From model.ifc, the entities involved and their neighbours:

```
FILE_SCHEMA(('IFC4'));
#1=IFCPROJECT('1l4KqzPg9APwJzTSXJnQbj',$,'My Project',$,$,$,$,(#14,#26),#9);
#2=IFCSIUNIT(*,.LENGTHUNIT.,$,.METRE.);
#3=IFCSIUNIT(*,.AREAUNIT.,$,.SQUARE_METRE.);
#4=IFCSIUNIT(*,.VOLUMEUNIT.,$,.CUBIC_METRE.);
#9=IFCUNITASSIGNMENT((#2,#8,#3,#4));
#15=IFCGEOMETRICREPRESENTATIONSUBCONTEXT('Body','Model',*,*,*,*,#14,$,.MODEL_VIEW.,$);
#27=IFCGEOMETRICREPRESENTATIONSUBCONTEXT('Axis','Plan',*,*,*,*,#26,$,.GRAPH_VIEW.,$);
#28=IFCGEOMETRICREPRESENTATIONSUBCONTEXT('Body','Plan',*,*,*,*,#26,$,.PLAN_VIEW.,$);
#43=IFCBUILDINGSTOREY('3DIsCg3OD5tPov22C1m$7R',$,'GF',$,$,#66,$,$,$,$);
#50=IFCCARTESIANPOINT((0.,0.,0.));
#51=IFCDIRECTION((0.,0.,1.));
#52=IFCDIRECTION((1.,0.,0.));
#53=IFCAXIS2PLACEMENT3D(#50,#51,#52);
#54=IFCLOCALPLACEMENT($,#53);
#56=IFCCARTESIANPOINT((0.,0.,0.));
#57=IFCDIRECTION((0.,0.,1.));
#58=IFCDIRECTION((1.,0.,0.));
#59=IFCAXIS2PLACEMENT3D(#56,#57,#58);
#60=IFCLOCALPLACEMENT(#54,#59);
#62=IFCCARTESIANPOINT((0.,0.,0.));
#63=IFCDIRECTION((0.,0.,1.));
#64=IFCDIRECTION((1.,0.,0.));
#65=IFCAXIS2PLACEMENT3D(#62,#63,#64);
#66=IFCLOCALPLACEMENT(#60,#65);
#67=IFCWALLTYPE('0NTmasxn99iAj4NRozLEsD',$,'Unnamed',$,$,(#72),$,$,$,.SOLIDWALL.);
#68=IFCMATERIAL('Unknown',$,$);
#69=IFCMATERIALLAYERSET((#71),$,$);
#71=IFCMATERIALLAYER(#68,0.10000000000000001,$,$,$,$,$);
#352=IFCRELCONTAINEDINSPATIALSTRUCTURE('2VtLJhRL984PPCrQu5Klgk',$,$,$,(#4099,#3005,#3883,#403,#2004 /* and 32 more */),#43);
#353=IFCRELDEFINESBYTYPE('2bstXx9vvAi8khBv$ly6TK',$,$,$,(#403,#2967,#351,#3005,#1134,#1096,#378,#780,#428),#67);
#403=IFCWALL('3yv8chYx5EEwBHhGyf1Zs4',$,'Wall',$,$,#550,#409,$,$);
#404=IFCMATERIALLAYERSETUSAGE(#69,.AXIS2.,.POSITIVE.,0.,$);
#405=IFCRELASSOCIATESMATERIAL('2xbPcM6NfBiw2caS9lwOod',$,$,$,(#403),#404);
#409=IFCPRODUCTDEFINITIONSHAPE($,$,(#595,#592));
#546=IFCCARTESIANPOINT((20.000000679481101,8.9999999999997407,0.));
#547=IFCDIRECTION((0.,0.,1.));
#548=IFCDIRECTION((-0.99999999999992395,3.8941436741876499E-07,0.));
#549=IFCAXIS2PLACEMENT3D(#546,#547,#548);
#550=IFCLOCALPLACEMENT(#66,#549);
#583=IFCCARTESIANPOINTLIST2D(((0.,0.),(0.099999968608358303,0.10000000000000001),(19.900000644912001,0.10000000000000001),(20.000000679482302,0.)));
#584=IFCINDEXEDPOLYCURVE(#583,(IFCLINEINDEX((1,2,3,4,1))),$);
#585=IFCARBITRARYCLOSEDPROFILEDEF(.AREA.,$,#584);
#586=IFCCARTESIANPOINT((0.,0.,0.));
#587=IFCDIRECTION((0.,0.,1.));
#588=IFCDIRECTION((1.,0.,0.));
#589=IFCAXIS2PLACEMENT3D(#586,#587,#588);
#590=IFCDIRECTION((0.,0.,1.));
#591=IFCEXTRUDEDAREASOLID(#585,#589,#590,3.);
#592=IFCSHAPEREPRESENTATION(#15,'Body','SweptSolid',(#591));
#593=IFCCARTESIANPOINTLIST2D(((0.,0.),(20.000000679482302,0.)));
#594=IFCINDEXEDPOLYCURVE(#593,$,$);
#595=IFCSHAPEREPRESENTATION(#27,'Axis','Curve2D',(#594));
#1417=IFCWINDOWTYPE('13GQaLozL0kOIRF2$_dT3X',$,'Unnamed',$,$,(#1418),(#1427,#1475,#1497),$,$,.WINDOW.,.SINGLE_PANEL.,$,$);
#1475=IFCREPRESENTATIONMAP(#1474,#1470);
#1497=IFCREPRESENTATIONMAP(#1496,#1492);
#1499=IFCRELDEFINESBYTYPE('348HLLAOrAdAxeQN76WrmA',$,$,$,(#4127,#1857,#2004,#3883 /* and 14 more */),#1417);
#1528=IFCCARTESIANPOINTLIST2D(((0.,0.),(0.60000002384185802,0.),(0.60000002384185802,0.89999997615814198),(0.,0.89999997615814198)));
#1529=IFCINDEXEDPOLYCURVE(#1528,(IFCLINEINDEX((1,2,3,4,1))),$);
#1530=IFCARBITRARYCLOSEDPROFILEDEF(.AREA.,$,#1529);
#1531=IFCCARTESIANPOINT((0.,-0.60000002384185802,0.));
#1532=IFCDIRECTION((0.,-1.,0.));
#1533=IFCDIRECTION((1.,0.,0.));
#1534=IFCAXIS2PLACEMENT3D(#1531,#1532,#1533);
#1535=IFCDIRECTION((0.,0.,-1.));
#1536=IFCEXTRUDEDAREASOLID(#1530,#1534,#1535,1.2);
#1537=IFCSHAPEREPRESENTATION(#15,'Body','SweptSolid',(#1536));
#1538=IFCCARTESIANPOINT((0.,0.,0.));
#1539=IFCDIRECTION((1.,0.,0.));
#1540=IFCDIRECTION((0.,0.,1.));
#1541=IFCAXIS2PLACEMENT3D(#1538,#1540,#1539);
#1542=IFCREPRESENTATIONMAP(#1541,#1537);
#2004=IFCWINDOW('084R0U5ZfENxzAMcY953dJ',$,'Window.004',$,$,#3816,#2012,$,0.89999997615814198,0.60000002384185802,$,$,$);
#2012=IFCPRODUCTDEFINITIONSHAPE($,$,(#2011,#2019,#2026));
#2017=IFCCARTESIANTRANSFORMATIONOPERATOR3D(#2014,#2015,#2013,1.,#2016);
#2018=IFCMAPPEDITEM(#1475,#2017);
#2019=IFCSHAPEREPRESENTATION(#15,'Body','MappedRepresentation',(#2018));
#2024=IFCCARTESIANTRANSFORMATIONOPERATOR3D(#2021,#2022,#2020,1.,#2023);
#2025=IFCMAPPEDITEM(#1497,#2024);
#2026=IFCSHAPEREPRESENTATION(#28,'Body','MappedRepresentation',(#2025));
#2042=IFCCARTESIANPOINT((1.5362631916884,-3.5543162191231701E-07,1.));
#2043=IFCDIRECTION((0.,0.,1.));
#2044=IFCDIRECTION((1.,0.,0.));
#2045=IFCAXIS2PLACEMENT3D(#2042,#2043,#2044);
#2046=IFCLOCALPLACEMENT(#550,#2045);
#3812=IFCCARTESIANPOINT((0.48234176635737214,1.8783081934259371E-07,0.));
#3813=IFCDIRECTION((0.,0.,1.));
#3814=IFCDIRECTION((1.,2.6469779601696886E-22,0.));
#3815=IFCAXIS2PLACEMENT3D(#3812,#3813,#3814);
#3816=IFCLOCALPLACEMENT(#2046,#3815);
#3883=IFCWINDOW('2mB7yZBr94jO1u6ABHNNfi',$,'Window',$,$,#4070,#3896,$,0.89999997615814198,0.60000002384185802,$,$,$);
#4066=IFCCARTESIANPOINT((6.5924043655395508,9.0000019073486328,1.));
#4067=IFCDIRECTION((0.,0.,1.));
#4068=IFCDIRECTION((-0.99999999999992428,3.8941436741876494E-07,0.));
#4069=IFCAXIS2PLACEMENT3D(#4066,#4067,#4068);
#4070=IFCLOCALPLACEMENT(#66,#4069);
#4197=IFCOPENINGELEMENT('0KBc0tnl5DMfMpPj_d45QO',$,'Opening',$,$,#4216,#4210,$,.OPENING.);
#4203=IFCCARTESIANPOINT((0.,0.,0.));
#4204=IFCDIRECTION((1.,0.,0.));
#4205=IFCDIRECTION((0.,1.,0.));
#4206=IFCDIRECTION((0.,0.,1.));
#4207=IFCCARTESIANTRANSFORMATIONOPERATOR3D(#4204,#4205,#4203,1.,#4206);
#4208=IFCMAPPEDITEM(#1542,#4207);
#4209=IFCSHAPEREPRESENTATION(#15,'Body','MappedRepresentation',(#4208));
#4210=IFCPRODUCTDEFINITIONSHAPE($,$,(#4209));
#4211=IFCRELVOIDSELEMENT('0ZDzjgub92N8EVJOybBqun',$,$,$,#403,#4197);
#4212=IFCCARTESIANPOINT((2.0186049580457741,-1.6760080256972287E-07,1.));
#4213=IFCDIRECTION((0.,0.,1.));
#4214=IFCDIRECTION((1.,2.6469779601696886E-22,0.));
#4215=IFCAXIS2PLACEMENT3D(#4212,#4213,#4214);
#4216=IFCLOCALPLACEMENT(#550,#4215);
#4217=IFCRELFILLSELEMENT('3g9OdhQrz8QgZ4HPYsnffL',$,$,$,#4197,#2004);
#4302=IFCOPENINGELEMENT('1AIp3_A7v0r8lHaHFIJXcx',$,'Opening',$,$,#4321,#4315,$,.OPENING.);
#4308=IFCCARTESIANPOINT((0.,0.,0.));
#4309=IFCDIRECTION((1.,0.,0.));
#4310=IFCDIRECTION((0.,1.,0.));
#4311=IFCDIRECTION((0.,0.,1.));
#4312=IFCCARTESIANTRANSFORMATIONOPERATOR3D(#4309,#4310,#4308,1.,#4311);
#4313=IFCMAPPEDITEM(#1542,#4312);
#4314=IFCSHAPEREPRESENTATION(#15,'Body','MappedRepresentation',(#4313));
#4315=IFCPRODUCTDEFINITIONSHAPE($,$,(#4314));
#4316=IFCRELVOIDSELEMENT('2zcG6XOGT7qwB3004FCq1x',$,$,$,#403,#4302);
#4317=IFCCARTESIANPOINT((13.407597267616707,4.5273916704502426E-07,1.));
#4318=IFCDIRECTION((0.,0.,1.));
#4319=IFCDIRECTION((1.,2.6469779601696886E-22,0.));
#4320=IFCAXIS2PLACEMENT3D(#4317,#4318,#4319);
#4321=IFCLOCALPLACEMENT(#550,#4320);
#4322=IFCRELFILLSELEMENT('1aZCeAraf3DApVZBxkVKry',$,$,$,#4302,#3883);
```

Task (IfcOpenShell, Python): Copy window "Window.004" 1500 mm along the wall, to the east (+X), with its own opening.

```python
import ifcopenshell
import ifcopenshell.api.feature
import ifcopenshell.api.geometry
import ifcopenshell.api.root
import ifcopenshell.geom
import ifcopenshell.util.element
import ifcopenshell.util.placement
import ifcopenshell.util.shape
import ifcopenshell.util.unit

model = ifcopenshell.open("model.ifc")
unit_scale = ifcopenshell.util.unit.calculate_unit_scale(model)
settings = ifcopenshell.geom.settings()


def volume(element):
    """Net volume in cubic metres, openings subtracted."""
    shape = ifcopenshell.geom.create_shape(settings, element)
    return ifcopenshell.util.shape.get_volume(shape.geometry)


window = model.by_guid("084R0U5ZfENxzAMcY953dJ")
opening = window.FillsVoids[0].RelatingOpeningElement
wall = opening.VoidsElements[0].RelatingBuildingElement
before = volume(wall)
shift = ifcopenshell.util.placement.get_local_placement(wall.ObjectPlacement)[:3, 0] * -1.5 / unit_scale

# copy_class copies the void relationship, type, container and properties, but no geometry.
new_opening = ifcopenshell.api.root.copy_class(model, product=opening)
new_opening.Representation = ifcopenshell.util.element.copy_deep(
    model, opening.Representation, exclude=["IfcGeometricRepresentationContext", "IfcRepresentationMap"]
)
new_window = ifcopenshell.api.root.copy_class(model, product=window)
new_window.Representation = ifcopenshell.util.element.copy_deep(
    model, window.Representation, exclude=["IfcGeometricRepresentationContext", "IfcRepresentationMap"]
)
ifcopenshell.api.feature.add_filling(model, opening=new_opening, element=new_window)

for old, new in ((opening, new_opening), (window, new_window)):
    matrix = ifcopenshell.util.placement.get_local_placement(old.ObjectPlacement)
    matrix[:3, 3] += shift
    ifcopenshell.api.geometry.edit_object_placement(model, product=new, matrix=matrix, is_si=False)

after = volume(wall)

print(f"wall volume {before:.3f} -> {after:.3f} m3")

model.write("model_v2.ifc")
```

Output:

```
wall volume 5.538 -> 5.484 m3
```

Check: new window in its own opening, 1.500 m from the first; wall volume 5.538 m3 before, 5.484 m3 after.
